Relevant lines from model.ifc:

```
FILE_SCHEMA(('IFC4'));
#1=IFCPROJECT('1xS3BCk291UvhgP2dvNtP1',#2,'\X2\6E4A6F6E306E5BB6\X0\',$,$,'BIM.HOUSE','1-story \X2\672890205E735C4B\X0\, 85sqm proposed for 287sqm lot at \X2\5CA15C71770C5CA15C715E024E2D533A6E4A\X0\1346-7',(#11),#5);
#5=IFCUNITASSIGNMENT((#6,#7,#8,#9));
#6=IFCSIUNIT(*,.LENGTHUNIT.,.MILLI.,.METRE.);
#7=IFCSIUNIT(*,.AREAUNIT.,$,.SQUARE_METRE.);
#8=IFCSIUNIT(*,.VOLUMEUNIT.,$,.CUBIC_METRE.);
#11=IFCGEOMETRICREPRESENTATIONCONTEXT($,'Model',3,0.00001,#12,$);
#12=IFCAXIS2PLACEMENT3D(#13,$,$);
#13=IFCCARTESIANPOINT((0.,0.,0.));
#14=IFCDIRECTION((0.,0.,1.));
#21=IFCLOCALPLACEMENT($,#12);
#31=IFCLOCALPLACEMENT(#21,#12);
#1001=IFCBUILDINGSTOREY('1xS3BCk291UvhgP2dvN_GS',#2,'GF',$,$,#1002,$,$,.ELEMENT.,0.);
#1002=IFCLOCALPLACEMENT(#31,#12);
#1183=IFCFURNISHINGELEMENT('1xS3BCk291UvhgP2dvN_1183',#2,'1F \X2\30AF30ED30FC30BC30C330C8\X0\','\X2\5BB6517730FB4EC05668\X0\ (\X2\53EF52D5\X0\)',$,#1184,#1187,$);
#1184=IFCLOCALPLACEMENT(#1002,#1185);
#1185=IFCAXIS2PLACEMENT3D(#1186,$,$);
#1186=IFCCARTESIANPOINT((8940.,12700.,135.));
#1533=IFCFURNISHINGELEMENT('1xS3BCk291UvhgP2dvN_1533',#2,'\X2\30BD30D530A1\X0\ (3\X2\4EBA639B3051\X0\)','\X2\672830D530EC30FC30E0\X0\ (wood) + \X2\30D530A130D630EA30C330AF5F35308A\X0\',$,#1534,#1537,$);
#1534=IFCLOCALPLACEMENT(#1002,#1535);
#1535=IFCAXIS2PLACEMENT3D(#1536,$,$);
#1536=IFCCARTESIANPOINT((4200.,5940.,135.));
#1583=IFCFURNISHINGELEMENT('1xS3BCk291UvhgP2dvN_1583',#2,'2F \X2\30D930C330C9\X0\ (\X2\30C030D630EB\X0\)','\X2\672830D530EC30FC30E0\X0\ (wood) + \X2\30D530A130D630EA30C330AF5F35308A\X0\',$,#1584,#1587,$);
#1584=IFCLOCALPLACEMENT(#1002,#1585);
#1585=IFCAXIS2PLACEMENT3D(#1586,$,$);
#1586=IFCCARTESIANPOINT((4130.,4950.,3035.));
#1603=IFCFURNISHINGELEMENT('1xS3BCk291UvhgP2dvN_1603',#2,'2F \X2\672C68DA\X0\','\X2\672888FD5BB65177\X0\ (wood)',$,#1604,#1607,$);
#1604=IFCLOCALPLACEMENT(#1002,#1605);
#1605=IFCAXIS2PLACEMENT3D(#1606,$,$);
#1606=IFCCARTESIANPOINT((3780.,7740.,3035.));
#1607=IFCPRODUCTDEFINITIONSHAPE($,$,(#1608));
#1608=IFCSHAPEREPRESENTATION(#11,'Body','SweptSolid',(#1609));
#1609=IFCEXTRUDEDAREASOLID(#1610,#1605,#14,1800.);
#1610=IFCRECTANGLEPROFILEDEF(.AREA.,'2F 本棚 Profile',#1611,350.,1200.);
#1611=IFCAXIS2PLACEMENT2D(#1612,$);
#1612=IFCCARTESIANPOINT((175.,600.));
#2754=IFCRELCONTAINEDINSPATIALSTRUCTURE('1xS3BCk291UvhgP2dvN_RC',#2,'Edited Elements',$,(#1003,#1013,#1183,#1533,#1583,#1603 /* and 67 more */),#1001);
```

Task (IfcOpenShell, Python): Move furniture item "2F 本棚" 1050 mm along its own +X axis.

```python
import ifcopenshell
import ifcopenshell.api.geometry
import ifcopenshell.util.placement

model = ifcopenshell.open("model.ifc")

item = model.by_id(1603)
matrix = ifcopenshell.util.placement.get_local_placement(item.ObjectPlacement)
matrix[:3, 3] += matrix[:3, 0] * 1050.0
ifcopenshell.api.geometry.edit_object_placement(model, product=item, matrix=matrix, is_si=False)

print(ifcopenshell.util.placement.get_local_placement(item.ObjectPlacement).round(3) + 0.0)

model.write("model_v2.ifc")
```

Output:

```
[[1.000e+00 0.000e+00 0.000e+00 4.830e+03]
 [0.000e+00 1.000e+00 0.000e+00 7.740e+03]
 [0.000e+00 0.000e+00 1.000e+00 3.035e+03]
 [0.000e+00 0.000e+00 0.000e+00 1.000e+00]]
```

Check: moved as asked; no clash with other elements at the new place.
